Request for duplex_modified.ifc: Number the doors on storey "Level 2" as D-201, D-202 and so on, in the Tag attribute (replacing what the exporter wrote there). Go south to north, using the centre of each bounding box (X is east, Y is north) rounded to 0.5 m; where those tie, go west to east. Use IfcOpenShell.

First a look at what the model holds.

```python
import ifcopenshell
import ifcopenshell.util.element
import ifcopenshell.util.placement

model = ifcopenshell.open("duplex_modified.ifc")
print(model.schema)
storey = next(s for s in model.by_type("IfcBuildingStorey") if s.Name == "Level 2")
doors = [e for e in ifcopenshell.util.element.get_decomposition(storey) if e.is_a("IfcDoor")]
for e in sorted(doors, key=lambda e: e.id()):
    origin = ifcopenshell.util.placement.get_local_placement(e.ObjectPlacement)[:3, 3]
    print(e.id(), e.Tag, e.Name, origin.round(2) + 0.0, sep=" | ")
```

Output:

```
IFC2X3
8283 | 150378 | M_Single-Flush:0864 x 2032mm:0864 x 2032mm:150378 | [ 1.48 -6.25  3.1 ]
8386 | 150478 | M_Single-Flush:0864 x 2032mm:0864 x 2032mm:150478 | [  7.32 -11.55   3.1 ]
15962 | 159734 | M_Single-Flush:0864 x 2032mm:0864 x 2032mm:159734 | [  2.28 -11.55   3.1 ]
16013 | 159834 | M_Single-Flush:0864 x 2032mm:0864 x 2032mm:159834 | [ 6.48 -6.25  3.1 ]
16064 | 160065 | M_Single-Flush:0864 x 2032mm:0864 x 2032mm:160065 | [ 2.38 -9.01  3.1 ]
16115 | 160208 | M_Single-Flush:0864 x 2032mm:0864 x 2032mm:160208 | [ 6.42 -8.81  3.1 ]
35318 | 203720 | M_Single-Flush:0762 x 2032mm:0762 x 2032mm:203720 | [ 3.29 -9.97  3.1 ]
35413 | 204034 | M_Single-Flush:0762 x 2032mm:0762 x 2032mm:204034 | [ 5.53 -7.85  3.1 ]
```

```python
import ifcopenshell
import ifcopenshell.geom
import ifcopenshell.util.element
import ifcopenshell.util.shape

model = ifcopenshell.open("duplex_modified.ifc")
settings = ifcopenshell.geom.settings()
settings.set("use-world-coords", True)


def centre(element):
    shape = ifcopenshell.geom.create_shape(settings, element)
    return ifcopenshell.util.shape.get_bbox_centroid(shape.geometry)


storey = next(s for s in model.by_type("IfcBuildingStorey") if s.Name == "Level 2")
doors = [e for e in ifcopenshell.util.element.get_decomposition(storey) if e.is_a("IfcDoor")]

# Insertion points can sit at a corner or the storey origin, so sort by the geometry (in metres).
centres = {e: centre(e) for e in doors}
doors.sort(key=lambda e: (round(centres[e][1] / 0.5), centres[e][0]))

for i, e in enumerate(doors, start=1):
    number = f"D-2{i:02d}"
    e.Tag = number
    print(e.id(), number)

model.write("duplex_modified-out.ifc")
```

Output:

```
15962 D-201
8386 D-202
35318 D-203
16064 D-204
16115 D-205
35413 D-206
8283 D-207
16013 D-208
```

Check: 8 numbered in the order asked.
